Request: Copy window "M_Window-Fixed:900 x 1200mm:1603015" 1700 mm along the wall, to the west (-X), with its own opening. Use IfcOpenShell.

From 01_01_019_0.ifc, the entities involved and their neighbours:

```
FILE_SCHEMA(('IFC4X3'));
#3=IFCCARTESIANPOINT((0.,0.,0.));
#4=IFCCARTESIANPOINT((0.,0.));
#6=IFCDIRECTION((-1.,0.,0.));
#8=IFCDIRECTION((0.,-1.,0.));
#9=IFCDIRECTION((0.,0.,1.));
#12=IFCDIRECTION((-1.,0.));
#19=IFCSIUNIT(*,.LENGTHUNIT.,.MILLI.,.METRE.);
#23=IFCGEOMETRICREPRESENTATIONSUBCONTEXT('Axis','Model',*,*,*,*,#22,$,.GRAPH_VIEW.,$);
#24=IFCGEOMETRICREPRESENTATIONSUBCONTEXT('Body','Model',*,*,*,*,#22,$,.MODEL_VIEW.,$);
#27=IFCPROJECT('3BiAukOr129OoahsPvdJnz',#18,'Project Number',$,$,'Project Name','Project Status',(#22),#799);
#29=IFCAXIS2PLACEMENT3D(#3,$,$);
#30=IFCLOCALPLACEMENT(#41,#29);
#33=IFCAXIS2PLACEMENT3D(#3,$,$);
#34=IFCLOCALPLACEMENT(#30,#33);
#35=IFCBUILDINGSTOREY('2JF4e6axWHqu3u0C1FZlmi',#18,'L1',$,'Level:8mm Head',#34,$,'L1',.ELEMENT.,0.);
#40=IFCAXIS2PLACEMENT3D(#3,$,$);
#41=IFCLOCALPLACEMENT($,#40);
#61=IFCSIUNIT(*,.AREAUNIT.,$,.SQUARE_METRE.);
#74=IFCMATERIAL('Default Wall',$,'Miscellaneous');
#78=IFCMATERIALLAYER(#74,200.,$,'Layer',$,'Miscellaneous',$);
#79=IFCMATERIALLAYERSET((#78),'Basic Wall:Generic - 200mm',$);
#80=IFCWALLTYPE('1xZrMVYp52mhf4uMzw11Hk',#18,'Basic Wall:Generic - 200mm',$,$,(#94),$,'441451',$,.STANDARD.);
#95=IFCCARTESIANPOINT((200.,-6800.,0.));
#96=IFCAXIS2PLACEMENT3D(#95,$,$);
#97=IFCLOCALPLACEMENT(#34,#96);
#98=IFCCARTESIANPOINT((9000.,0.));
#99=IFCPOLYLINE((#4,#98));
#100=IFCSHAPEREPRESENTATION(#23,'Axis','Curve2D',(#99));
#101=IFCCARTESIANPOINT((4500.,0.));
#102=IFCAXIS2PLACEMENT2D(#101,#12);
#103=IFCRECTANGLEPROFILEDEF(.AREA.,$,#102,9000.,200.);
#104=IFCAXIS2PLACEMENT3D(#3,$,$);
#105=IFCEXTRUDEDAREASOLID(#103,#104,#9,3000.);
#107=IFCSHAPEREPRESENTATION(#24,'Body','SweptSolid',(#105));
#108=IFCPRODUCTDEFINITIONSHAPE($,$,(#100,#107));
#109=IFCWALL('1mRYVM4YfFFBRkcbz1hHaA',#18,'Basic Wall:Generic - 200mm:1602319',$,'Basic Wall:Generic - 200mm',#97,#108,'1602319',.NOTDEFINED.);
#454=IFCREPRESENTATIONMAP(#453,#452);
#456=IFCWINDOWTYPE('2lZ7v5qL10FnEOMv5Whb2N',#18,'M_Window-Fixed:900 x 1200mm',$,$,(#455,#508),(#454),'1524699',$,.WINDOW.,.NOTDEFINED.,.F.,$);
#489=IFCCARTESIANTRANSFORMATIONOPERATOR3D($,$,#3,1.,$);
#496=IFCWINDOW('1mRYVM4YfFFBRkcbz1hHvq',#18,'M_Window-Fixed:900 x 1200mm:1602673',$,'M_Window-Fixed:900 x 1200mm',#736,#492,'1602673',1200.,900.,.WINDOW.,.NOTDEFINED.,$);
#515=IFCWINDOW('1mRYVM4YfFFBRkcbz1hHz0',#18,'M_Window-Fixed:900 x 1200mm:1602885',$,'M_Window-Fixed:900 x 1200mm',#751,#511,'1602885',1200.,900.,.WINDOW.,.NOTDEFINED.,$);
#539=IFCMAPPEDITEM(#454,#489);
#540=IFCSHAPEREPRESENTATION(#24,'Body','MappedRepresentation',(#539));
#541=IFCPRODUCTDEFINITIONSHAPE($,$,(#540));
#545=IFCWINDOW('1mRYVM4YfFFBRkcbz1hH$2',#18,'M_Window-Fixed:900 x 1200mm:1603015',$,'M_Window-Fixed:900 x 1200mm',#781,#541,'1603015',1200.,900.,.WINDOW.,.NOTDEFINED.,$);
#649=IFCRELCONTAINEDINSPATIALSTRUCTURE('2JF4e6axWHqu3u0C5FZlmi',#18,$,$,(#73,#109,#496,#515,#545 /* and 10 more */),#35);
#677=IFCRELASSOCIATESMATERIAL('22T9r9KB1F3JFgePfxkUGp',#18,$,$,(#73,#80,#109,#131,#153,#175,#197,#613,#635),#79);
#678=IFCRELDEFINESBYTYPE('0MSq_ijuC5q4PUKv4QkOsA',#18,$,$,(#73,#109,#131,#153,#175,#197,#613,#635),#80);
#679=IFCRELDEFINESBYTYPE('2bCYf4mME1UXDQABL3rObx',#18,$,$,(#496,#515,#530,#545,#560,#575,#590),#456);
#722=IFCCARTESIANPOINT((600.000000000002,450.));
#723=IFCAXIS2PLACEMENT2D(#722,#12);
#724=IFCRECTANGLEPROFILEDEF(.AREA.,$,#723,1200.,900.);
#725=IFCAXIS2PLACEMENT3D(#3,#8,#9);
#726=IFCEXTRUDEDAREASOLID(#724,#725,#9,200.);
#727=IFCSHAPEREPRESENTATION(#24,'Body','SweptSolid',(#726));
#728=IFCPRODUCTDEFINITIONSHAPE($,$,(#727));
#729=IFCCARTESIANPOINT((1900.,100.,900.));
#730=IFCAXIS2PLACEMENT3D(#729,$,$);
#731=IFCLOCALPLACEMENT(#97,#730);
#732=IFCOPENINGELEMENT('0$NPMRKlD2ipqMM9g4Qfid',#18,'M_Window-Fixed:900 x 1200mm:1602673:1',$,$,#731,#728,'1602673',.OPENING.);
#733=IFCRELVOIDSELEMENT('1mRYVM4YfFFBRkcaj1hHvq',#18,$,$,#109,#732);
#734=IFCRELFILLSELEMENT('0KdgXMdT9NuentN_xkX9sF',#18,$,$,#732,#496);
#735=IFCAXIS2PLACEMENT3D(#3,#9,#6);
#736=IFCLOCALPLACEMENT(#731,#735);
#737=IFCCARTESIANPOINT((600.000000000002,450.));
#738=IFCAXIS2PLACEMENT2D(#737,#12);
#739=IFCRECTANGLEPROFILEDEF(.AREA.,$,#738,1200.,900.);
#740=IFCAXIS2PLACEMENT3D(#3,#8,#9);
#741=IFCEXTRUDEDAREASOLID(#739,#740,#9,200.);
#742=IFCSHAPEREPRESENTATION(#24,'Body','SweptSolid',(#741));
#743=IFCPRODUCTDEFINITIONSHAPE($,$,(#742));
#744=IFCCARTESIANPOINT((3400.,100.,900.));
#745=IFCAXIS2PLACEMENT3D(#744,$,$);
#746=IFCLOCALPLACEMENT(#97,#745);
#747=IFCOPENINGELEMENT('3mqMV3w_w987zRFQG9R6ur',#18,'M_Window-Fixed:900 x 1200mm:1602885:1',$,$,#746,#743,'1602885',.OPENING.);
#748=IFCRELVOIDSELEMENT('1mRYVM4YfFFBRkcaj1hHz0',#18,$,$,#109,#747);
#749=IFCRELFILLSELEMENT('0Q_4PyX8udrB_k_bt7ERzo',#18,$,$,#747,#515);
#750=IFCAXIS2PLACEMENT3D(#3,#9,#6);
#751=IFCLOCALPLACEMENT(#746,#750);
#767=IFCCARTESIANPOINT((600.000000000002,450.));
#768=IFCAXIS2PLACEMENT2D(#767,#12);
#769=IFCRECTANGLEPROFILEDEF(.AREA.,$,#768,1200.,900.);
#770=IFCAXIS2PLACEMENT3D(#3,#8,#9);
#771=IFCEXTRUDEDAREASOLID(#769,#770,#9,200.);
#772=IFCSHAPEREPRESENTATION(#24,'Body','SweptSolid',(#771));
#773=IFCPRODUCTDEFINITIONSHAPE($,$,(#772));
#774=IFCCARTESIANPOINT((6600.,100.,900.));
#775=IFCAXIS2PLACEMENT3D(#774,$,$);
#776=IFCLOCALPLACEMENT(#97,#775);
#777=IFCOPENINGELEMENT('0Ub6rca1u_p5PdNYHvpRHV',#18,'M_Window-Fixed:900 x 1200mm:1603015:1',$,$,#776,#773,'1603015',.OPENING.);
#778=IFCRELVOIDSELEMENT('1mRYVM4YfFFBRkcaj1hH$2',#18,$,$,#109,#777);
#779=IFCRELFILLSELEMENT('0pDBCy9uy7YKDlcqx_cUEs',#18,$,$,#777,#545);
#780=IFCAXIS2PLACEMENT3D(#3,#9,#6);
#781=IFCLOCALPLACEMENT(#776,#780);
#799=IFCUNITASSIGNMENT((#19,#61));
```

```python
import ifcopenshell
import ifcopenshell.api.feature
import ifcopenshell.api.geometry
import ifcopenshell.api.root
import ifcopenshell.geom
import ifcopenshell.util.element
import ifcopenshell.util.placement
import ifcopenshell.util.shape
import ifcopenshell.util.unit

model = ifcopenshell.open("01_01_019_0.ifc")
unit_scale = ifcopenshell.util.unit.calculate_unit_scale(model)
settings = ifcopenshell.geom.settings()


def volume(element):
    """Net volume in cubic metres, openings subtracted."""
    shape = ifcopenshell.geom.create_shape(settings, element)
    return ifcopenshell.util.shape.get_volume(shape.geometry)


def reuse_history(source, copy):
    """copy_class also copies each property set's owner history, people and application; keep the originals."""
    for rel in copy.IsDefinedBy:
        if rel.is_a("IfcRelDefinesByProperties") and (history := rel.RelatingPropertyDefinition.OwnerHistory):
            rel.RelatingPropertyDefinition.OwnerHistory = source.OwnerHistory
            ifcopenshell.util.element.remove_deep2(model, history)


window = model.by_guid("1mRYVM4YfFFBRkcbz1hH$2")
opening = window.FillsVoids[0].RelatingOpeningElement
wall = opening.VoidsElements[0].RelatingBuildingElement
before = volume(wall)
shift = ifcopenshell.util.placement.get_local_placement(wall.ObjectPlacement)[:3, 0] * -1.7 / unit_scale

# copy_class copies the void relationship, type, container and properties, but no geometry.
new_opening = ifcopenshell.api.root.copy_class(model, product=opening)
new_opening.Representation = ifcopenshell.util.element.copy_deep(
    model, opening.Representation, exclude=["IfcGeometricRepresentationContext", "IfcRepresentationMap"]
)
new_opening.Name = "M_Window-Fixed:900 x 1200mm"
new_opening.Tag = None
new_window = ifcopenshell.api.root.copy_class(model, product=window)
new_window.Representation = ifcopenshell.util.element.copy_deep(
    model, window.Representation, exclude=["IfcGeometricRepresentationContext", "IfcRepresentationMap"]
)
new_window.Name = "M_Window-Fixed:900 x 1200mm"
new_window.Tag = None
reuse_history(window, new_window)
ifcopenshell.api.feature.add_filling(model, opening=new_opening, element=new_window)

for old, new in ((opening, new_opening), (window, new_window)):
    matrix = ifcopenshell.util.placement.get_local_placement(old.ObjectPlacement)
    matrix[:3, 3] += shift
    ifcopenshell.api.geometry.edit_object_placement(model, product=new, matrix=matrix, is_si=False)

after = volume(wall)

print(f"wall volume {before:.3f} -> {after:.3f} m3")

model.write("01_01_019_0_v2.ifc")
```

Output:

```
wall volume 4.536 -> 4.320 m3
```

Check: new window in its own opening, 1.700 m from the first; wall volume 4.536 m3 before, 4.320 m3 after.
